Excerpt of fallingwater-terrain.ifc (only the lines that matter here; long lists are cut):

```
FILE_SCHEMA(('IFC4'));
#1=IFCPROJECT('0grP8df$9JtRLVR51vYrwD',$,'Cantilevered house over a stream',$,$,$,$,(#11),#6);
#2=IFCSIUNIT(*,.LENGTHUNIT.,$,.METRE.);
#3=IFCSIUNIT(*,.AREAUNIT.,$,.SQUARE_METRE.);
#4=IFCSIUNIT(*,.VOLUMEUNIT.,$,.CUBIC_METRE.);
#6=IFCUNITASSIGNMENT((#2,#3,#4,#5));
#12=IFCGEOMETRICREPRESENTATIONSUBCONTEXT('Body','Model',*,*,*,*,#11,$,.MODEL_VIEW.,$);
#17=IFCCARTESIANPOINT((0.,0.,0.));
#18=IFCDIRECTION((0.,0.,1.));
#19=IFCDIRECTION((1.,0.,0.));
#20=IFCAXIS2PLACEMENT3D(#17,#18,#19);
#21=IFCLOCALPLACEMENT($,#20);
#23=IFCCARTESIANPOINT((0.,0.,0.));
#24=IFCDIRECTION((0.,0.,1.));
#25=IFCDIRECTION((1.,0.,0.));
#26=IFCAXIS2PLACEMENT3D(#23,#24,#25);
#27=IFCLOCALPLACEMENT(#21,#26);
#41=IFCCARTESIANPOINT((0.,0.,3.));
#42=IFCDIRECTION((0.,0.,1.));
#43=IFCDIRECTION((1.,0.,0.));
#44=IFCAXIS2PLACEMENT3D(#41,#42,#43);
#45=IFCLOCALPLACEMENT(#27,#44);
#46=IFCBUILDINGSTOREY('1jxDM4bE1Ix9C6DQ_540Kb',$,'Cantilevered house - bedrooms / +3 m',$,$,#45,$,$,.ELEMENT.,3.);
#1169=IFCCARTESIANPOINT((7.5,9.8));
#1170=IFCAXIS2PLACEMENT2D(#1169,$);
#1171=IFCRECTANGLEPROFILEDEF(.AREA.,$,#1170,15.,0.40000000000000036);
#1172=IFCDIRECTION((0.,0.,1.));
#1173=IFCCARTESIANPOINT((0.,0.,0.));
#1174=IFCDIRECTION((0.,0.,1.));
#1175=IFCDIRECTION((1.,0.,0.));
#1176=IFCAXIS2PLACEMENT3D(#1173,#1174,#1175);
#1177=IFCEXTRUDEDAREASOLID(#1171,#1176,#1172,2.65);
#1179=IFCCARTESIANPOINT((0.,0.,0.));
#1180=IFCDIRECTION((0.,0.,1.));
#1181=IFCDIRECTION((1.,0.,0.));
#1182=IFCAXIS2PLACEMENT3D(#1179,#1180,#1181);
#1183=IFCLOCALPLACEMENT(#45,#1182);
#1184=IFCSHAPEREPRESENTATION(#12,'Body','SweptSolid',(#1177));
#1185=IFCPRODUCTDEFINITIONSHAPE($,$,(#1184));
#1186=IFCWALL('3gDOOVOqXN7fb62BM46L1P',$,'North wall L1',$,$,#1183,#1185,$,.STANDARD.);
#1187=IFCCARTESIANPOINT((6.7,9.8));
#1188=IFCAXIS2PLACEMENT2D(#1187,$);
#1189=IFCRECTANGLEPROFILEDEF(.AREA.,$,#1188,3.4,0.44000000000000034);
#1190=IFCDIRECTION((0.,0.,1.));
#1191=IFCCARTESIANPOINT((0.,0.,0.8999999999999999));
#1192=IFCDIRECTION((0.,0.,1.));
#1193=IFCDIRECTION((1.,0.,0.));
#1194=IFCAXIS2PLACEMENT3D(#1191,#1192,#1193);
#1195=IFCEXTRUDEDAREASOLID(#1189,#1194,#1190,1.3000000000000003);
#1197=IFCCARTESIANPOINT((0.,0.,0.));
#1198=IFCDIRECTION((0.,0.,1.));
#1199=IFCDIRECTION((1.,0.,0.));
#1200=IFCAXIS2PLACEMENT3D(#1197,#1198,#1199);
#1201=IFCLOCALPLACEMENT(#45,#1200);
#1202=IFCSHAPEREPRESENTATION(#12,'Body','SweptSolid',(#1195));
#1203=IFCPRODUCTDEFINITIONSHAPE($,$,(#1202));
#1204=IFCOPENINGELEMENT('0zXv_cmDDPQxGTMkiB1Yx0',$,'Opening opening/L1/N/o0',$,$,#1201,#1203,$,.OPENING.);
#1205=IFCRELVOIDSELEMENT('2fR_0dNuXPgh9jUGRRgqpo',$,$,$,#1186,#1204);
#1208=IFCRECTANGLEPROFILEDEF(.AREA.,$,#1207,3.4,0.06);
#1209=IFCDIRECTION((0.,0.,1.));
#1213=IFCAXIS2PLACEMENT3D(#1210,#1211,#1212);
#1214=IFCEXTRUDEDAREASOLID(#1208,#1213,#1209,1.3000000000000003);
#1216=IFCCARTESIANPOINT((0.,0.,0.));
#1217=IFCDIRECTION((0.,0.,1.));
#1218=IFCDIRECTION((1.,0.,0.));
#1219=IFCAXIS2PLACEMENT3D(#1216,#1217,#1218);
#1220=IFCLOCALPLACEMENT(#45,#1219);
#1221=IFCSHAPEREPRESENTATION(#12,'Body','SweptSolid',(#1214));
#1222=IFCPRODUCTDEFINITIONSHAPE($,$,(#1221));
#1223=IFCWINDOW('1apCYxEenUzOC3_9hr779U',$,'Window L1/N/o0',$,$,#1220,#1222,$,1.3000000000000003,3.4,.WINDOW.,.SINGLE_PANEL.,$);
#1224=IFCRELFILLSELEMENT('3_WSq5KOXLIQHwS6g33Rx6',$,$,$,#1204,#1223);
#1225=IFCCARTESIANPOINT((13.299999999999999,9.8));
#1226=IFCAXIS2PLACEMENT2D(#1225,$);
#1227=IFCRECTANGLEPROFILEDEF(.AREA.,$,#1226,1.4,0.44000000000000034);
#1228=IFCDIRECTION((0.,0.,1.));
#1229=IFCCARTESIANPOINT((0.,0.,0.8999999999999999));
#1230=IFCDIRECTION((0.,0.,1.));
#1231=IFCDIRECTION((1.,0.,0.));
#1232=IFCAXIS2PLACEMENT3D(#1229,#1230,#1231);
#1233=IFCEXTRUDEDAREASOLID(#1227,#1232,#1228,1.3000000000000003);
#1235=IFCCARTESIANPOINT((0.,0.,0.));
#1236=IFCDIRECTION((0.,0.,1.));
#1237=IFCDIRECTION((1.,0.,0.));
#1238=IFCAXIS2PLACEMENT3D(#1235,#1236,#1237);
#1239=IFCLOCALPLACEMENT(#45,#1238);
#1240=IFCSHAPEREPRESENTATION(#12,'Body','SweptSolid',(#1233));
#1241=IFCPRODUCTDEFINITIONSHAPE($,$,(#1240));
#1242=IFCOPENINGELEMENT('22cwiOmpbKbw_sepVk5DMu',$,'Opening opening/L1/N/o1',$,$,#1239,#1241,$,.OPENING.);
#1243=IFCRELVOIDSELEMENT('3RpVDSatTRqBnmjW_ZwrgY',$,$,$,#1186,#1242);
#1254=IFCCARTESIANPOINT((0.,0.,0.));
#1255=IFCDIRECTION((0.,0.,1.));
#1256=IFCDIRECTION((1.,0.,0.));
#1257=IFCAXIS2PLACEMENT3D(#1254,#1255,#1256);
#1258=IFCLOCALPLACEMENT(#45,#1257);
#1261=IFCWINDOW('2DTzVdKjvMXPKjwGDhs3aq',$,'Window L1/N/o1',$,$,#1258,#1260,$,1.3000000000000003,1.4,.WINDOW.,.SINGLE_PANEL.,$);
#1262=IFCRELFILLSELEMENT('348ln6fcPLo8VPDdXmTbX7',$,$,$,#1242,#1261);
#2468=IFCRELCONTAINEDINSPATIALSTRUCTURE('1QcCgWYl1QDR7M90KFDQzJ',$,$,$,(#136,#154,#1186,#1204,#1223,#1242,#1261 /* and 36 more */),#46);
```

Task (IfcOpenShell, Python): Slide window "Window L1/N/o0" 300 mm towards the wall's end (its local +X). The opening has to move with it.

```python
import ifcopenshell
import ifcopenshell.api.geometry
import ifcopenshell.util.placement
import ifcopenshell.util.unit

model = ifcopenshell.open("fallingwater-terrain.ifc")
unit_scale = ifcopenshell.util.unit.calculate_unit_scale(model)

window = model.by_id(1223)
opening = window.FillsVoids[0].RelatingOpeningElement
wall = opening.VoidsElements[0].RelatingBuildingElement

wall_matrix = ifcopenshell.util.placement.get_local_placement(wall.ObjectPlacement)
shift = wall_matrix[:3, 0] * 0.3 / unit_scale
before = ifcopenshell.util.placement.get_local_placement(window.ObjectPlacement)[:3, 3].copy()

# The window is not placed relative to its opening, so move both.
for product in (opening, window):
    matrix = ifcopenshell.util.placement.get_local_placement(product.ObjectPlacement)
    matrix[:3, 3] += shift
    ifcopenshell.api.geometry.edit_object_placement(model, product=product, matrix=matrix, is_si=False)

after = ifcopenshell.util.placement.get_local_placement(window.ObjectPlacement)[:3, 3]
print("window moved by", (after - before).round(3) + 0.0)

model.write("fallingwater-terrain-out.ifc")
```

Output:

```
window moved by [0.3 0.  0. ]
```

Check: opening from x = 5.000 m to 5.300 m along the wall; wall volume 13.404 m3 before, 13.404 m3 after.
